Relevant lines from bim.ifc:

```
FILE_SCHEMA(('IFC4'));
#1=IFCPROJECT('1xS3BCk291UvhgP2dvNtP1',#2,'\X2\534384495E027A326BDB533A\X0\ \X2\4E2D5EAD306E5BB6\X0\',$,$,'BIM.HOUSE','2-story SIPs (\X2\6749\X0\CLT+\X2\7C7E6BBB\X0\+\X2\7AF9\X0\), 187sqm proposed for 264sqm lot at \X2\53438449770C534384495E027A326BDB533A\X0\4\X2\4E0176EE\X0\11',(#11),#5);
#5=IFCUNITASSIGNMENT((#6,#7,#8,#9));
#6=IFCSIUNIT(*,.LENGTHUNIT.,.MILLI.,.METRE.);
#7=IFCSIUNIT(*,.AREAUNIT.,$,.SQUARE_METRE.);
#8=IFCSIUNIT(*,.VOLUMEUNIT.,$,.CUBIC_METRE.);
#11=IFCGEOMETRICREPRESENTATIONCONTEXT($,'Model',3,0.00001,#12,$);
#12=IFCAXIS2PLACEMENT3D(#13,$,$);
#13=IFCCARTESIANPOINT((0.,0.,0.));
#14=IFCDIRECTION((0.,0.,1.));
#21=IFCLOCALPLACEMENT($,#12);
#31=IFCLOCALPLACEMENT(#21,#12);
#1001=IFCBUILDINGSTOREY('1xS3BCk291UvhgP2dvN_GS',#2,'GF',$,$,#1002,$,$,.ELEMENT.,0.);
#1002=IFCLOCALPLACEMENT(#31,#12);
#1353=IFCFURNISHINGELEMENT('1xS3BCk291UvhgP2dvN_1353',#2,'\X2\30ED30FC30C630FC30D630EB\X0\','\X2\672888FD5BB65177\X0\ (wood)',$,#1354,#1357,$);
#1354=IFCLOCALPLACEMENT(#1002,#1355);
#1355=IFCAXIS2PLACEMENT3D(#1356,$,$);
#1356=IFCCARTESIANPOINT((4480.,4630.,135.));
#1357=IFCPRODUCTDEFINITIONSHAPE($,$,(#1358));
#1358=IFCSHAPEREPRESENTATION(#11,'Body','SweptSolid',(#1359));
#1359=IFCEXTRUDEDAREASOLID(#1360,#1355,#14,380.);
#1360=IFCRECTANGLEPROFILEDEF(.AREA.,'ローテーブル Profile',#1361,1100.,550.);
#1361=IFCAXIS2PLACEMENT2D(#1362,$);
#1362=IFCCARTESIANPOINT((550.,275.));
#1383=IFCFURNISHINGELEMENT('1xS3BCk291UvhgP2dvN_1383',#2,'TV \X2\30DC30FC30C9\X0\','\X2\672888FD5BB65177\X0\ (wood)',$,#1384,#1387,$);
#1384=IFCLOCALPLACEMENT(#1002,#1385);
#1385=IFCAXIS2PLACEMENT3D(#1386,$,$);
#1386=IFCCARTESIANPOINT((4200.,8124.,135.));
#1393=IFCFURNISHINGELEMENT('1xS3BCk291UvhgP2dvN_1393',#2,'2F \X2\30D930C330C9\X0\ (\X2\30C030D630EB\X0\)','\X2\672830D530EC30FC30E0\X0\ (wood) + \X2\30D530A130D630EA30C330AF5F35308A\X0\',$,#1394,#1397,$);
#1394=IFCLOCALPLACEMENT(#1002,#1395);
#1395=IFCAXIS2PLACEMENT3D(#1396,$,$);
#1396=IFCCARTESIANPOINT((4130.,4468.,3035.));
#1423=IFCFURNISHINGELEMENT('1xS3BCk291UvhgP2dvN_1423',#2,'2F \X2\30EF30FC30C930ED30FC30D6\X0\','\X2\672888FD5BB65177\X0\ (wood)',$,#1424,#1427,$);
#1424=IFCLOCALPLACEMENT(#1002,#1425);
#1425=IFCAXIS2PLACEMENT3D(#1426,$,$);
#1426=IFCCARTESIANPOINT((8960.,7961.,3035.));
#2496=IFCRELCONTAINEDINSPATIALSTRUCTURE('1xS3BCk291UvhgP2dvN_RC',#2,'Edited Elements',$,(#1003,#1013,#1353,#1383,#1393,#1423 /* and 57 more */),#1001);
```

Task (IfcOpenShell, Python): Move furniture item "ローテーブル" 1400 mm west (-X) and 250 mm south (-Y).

```python
import ifcopenshell
import ifcopenshell.api.geometry
import ifcopenshell.util.placement
import ifcopenshell.util.unit

model = ifcopenshell.open("bim.ifc")
unit_scale = ifcopenshell.util.unit.calculate_unit_scale(model)

item = model.by_guid("1xS3BCk291UvhgP2dvN_1353")
matrix = ifcopenshell.util.placement.get_local_placement(item.ObjectPlacement)
matrix[0, 3] -= 1.4 / unit_scale
matrix[1, 3] -= 0.25 / unit_scale
ifcopenshell.api.geometry.edit_object_placement(model, product=item, matrix=matrix, is_si=False)

print(ifcopenshell.util.placement.get_local_placement(item.ObjectPlacement).round(3) + 0.0)

model.write("bim_v2.ifc")
```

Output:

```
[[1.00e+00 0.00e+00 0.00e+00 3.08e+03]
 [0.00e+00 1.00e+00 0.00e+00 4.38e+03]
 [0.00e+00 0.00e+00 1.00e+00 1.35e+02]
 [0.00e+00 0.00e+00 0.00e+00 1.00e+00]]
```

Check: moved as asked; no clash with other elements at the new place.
